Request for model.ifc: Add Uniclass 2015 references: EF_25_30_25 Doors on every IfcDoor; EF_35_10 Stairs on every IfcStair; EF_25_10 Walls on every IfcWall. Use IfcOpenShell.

First a look at what the model holds.

```python
import ifcopenshell

model = ifcopenshell.open("model.ifc")
print(model.schema)
print("classifications:", [c.Name for c in model.by_type("IfcClassification")])
for ifc_class in ("IfcDoor", "IfcRoof", "IfcStair", "IfcWall", "IfcWindow"):
    print(ifc_class, len(model.by_type(ifc_class)))
```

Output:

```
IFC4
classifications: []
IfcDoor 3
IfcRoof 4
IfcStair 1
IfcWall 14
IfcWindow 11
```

```python
import ifcopenshell
import ifcopenshell.api.classification

model = ifcopenshell.open("model.ifc")

system = ifcopenshell.api.classification.add_classification(model, classification="Uniclass 2015")

codes = {
    "IfcDoor": ("EF_25_30_25", "Doors"),
    "IfcStair": ("EF_35_10", "Stairs"),
    "IfcWall": ("EF_25_10", "Walls"),
}
for ifc_class, (code, name) in codes.items():
    products = model.by_type(ifc_class)
    ifcopenshell.api.classification.add_reference(
        model, products=products, classification=system, identification=code, name=name
    )
    print(code, len(products))

model.write("model-out.ifc")
```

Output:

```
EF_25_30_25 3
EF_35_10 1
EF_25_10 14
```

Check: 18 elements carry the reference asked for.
